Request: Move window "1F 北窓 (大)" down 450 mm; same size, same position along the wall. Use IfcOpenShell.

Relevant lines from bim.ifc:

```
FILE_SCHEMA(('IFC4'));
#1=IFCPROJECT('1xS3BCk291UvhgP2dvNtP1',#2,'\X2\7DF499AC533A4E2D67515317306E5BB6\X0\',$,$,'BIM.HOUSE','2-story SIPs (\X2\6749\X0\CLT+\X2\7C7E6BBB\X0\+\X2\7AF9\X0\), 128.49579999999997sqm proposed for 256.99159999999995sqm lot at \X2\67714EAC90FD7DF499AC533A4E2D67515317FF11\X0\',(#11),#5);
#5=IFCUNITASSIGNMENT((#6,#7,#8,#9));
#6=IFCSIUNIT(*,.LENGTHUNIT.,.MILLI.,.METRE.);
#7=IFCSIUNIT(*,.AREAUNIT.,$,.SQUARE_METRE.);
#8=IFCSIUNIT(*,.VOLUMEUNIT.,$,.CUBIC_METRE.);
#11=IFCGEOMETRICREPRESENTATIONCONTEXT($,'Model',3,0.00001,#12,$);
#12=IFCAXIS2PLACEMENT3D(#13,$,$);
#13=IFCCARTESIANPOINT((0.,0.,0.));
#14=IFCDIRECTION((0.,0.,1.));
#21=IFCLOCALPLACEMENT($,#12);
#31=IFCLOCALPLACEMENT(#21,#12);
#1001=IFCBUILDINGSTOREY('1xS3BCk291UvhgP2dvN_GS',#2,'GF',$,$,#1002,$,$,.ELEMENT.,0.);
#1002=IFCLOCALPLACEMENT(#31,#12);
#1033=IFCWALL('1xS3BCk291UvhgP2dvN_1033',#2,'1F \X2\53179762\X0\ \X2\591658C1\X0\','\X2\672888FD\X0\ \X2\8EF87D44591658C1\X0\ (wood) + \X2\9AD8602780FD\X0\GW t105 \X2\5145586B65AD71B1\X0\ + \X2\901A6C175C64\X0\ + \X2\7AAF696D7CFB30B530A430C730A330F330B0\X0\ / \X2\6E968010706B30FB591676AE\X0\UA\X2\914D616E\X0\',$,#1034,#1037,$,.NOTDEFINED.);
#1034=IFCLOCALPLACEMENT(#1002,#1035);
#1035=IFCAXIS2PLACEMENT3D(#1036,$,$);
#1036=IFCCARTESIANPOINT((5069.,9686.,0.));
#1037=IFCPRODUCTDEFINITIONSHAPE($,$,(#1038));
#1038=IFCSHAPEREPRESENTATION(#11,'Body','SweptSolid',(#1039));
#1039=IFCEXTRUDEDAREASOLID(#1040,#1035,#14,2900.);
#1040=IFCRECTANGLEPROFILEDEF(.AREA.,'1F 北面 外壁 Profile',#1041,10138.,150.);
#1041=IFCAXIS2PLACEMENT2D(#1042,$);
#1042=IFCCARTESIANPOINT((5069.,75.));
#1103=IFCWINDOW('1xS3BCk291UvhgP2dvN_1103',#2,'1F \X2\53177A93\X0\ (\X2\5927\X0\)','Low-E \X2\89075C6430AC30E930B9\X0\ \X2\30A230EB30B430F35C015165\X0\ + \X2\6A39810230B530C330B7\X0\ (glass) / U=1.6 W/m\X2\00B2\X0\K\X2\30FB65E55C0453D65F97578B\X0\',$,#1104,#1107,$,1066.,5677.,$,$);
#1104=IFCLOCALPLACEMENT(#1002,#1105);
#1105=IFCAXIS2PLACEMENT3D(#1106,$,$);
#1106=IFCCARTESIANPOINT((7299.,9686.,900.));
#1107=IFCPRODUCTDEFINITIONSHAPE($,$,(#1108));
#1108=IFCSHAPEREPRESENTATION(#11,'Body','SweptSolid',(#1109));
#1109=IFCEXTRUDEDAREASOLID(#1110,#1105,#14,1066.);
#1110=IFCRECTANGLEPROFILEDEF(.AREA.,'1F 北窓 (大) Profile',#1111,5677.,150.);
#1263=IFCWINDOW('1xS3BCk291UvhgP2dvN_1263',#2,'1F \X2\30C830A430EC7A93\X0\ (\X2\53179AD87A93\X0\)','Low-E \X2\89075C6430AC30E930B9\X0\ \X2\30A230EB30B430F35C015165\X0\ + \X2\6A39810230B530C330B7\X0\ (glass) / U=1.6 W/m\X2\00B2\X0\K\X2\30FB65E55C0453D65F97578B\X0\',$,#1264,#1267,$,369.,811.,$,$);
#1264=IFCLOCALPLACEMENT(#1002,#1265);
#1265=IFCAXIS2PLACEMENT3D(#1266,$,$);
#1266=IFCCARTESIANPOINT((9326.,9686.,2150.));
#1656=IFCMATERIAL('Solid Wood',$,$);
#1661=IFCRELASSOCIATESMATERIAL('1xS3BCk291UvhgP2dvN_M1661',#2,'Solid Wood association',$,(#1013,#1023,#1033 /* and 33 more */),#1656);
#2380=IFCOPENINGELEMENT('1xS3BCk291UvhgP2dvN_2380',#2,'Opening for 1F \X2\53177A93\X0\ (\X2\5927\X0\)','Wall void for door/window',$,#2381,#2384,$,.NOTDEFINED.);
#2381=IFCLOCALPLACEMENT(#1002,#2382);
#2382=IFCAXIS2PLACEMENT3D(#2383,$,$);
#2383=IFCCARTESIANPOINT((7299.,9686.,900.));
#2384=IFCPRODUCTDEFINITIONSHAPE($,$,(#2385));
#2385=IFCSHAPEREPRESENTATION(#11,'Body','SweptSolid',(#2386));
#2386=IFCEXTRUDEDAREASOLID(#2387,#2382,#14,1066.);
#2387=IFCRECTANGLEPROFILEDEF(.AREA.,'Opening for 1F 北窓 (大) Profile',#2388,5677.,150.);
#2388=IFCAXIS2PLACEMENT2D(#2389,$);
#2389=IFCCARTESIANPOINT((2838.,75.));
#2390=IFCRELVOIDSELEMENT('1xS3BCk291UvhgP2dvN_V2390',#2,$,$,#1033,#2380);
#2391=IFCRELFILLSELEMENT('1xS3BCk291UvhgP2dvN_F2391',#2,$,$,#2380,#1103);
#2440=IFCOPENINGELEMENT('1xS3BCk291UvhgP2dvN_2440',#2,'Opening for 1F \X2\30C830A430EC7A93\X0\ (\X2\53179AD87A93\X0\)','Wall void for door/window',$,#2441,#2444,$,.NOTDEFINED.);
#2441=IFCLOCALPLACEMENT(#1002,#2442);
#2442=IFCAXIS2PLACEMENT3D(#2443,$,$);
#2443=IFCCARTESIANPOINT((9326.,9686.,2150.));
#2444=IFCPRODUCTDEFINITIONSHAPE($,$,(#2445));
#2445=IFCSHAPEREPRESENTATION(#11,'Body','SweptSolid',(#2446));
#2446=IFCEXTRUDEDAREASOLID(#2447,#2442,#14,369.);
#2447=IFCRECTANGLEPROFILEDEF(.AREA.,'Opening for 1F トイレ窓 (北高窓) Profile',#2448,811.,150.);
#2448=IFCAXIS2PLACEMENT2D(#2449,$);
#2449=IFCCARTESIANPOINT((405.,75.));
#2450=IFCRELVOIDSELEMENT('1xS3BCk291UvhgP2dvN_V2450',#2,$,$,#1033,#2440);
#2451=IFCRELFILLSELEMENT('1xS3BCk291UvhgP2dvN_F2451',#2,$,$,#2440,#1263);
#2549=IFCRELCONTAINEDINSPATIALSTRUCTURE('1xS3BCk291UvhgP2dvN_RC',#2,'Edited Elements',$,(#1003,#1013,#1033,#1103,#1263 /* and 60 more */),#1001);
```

```python
import numpy as np
import ifcopenshell
import ifcopenshell.api.geometry
import ifcopenshell.util.placement
import ifcopenshell.util.unit

model = ifcopenshell.open("bim.ifc")
unit_scale = ifcopenshell.util.unit.calculate_unit_scale(model)

window = model.by_id(1103)
opening = window.FillsVoids[0].RelatingOpeningElement
dz = -0.45 / unit_scale

shift = np.array([0.0, 0.0, dz])
# The window is not placed relative to its opening, so move both.
for product in (opening, window):
    matrix = ifcopenshell.util.placement.get_local_placement(product.ObjectPlacement)
    matrix[:3, 3] += shift
    ifcopenshell.api.geometry.edit_object_placement(model, product=product, matrix=matrix, is_si=False)

print(f"moved by {dz * unit_scale:+.3f} m")

model.write("bim-out.ifc")
```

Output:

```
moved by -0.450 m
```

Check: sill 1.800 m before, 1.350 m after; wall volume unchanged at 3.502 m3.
